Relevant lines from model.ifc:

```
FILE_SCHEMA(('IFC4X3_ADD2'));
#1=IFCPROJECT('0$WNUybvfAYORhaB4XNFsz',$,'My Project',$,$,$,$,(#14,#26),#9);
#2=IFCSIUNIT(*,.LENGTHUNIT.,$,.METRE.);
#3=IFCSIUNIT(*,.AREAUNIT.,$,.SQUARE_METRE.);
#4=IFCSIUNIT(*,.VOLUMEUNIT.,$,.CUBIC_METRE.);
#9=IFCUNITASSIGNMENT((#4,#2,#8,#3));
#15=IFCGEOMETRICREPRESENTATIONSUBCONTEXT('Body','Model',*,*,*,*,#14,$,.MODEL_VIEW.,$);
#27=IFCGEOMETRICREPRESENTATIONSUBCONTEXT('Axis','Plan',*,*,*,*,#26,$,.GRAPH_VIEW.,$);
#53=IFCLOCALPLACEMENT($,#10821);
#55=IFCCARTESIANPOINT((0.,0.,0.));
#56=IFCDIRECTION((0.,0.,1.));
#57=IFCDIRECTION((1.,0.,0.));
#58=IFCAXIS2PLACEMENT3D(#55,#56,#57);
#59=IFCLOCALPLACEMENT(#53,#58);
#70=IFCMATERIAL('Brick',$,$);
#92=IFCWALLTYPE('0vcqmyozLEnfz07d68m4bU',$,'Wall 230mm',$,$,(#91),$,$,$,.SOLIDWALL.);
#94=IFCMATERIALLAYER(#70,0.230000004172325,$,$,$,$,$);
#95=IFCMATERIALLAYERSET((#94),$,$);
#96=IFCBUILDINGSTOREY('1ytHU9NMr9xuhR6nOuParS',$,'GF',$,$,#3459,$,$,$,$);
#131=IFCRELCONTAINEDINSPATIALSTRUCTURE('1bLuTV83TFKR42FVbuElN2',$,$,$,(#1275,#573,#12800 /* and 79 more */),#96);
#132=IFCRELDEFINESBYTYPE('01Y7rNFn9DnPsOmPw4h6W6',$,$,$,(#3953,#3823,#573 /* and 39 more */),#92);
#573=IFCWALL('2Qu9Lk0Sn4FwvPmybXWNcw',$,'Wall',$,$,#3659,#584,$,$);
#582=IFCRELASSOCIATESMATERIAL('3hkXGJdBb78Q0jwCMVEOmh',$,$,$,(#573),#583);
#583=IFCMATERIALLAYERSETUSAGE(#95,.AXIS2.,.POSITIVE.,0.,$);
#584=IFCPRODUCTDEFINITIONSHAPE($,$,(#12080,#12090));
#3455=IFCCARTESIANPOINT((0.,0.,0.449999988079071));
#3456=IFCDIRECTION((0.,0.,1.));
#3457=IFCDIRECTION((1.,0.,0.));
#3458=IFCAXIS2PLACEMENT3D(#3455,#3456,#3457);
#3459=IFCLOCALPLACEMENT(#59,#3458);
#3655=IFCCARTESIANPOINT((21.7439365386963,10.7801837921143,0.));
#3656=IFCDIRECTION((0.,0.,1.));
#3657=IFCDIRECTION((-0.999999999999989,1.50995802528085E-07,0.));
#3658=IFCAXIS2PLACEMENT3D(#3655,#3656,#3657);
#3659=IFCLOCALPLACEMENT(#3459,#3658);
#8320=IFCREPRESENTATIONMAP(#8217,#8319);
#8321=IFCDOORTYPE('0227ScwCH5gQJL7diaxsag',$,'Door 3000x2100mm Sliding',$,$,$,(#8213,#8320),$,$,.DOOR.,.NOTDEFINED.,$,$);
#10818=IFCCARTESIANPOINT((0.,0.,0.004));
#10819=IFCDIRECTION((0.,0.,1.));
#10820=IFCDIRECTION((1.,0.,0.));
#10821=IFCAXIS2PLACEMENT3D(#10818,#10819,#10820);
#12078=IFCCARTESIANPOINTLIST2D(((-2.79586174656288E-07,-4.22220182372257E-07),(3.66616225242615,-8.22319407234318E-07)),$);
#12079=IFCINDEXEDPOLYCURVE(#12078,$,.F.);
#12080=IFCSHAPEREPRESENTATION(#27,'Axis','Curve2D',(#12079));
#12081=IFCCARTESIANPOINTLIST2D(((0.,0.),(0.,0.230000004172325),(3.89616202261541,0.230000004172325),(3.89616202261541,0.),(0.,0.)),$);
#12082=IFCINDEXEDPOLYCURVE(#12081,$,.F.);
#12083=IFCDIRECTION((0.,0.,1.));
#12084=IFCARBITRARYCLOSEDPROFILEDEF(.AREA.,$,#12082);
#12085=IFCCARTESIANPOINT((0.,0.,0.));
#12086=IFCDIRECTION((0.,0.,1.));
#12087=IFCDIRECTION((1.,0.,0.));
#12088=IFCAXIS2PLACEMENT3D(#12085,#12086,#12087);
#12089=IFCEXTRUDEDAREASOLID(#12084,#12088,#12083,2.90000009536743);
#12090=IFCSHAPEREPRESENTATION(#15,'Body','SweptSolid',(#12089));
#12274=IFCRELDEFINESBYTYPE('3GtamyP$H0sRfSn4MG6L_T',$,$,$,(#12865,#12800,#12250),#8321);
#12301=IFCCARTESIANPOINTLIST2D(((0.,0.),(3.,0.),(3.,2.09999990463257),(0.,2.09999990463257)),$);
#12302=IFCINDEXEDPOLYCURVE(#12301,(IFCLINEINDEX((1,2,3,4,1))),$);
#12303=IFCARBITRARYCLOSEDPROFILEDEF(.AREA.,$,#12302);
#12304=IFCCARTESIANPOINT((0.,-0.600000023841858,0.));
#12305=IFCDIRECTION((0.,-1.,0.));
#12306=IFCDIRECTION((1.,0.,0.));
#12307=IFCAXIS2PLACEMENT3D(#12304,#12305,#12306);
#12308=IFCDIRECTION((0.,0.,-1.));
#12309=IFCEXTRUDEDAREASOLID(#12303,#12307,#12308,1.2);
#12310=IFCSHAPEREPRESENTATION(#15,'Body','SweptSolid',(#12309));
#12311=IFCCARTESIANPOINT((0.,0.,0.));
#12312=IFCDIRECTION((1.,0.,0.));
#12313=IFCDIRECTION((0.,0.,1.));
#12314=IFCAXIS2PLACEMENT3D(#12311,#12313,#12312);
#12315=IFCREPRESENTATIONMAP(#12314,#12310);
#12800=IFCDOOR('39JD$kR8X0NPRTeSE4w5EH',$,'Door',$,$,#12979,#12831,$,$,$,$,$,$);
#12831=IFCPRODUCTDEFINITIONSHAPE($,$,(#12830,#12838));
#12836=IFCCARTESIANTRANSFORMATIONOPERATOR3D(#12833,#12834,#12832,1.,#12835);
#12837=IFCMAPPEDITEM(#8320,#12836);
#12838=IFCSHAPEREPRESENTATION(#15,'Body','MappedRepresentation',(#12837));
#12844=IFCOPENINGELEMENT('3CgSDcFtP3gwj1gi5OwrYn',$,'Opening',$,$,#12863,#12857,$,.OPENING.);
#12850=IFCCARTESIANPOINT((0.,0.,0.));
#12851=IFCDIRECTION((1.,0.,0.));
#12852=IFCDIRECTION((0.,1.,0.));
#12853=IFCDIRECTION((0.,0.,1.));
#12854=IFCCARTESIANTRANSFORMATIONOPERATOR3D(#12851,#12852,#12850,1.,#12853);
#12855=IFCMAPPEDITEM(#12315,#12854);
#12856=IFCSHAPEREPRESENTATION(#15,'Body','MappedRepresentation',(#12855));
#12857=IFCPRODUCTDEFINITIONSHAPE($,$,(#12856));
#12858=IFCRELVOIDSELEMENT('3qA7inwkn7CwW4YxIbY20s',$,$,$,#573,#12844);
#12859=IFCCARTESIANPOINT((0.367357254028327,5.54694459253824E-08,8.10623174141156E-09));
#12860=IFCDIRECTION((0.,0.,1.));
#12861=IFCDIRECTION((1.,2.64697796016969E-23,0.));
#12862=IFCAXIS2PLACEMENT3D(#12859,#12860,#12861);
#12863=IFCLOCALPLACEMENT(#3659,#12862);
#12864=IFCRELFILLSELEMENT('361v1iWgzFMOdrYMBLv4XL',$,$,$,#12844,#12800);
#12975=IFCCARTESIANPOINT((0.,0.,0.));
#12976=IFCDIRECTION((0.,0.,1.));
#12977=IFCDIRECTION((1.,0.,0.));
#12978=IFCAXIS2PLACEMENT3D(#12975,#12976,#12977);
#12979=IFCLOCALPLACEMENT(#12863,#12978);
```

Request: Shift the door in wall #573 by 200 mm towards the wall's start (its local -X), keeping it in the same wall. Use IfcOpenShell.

```python
import ifcopenshell
import ifcopenshell.api.geometry
import ifcopenshell.util.placement
import ifcopenshell.util.unit

model = ifcopenshell.open("model.ifc")
unit_scale = ifcopenshell.util.unit.calculate_unit_scale(model)

door = model.by_guid("39JD$kR8X0NPRTeSE4w5EH")
opening = door.FillsVoids[0].RelatingOpeningElement
wall = opening.VoidsElements[0].RelatingBuildingElement

wall_matrix = ifcopenshell.util.placement.get_local_placement(wall.ObjectPlacement)
shift = wall_matrix[:3, 0] * -0.2 / unit_scale
before = ifcopenshell.util.placement.get_local_placement(door.ObjectPlacement)[:3, 3].copy()

# The door is placed relative to its opening, so it follows when the opening moves.
matrix = ifcopenshell.util.placement.get_local_placement(opening.ObjectPlacement)
matrix[:3, 3] += shift
ifcopenshell.api.geometry.edit_object_placement(
    model, product=opening, matrix=matrix, is_si=False, should_transform_children=True
)

after = ifcopenshell.util.placement.get_local_placement(door.ObjectPlacement)[:3, 3]
print("door moved by", (after - before).round(3) + 0.0)

model.write("model_updated.ifc")
```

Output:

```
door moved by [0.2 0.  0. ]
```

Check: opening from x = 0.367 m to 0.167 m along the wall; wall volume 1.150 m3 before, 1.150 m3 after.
